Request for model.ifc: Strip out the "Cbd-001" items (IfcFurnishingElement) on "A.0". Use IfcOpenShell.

First a look at what the model holds.

```python
import ifcopenshell
import ifcopenshell.util.element

model = ifcopenshell.open("model.ifc")
print(model.schema)
storey = next(s for s in model.by_type("IfcBuildingStorey") if s.Name == "A.0")
furniture = [e for e in ifcopenshell.util.element.get_decomposition(storey) if e.is_a("IfcFurnishingElement")]
seen = {}
for e in furniture:
    element_type = ifcopenshell.util.element.get_type(e)
    name = element_type.Name if element_type not in (None, e) else None
    seen[name] = seen.get(name, 0) + 1
for name, count in sorted(seen.items(), key=str):
    print(count, "x", name)
```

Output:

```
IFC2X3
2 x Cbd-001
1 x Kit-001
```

```python
import ifcopenshell
import ifcopenshell.api.root
import ifcopenshell.util.element

model = ifcopenshell.open("model.ifc")

storey = next(s for s in model.by_type("IfcBuildingStorey") if s.Name == "A.0")
furniture = [e for e in ifcopenshell.util.element.get_decomposition(storey) if e.is_a("IfcFurnishingElement")]
targets = [e for e in furniture if (t := ifcopenshell.util.element.get_type(e)) not in (None, e) and t.Name == "Cbd-001"]

for e in targets:
    ifcopenshell.api.root.remove_product(model, product=e)
print(len(targets), "removed")

model.write("model_rev.ifc")
```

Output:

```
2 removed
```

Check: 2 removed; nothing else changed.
